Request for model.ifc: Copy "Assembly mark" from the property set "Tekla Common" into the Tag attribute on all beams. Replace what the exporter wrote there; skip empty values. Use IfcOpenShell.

First a look at what the model holds.

```python
import ifcopenshell
import ifcopenshell.util.element

model = ifcopenshell.open("model.ifc")
print(model.schema)
beams = model.by_type("IfcBeam")
print(len(beams), "beams")
for e in beams[:8]:
    source = ifcopenshell.util.element.get_pset(e, "Tekla Common", "Assembly mark")
    target = e.Tag
    print(e.id(), repr(source), repr(target), sep=" | ")
```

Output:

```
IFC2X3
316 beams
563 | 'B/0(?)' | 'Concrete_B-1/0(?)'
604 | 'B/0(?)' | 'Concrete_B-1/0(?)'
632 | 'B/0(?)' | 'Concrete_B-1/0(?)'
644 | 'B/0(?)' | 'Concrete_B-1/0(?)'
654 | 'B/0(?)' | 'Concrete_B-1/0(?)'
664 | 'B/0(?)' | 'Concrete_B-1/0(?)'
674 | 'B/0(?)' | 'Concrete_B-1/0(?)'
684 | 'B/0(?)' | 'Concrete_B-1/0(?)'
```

```python
import ifcopenshell
import ifcopenshell.util.element

model = ifcopenshell.open("model.ifc")

count = 0
for e in model.by_type("IfcBeam"):
    value = ifcopenshell.util.element.get_pset(e, "Tekla Common", "Assembly mark")
    current = e.Tag
    if not value or not value.strip() or current == value:
        continue
    e.Tag = value
    count += 1

print(count, "beams updated")

model.write("model_rev.ifc")
```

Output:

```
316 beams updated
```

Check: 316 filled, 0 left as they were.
